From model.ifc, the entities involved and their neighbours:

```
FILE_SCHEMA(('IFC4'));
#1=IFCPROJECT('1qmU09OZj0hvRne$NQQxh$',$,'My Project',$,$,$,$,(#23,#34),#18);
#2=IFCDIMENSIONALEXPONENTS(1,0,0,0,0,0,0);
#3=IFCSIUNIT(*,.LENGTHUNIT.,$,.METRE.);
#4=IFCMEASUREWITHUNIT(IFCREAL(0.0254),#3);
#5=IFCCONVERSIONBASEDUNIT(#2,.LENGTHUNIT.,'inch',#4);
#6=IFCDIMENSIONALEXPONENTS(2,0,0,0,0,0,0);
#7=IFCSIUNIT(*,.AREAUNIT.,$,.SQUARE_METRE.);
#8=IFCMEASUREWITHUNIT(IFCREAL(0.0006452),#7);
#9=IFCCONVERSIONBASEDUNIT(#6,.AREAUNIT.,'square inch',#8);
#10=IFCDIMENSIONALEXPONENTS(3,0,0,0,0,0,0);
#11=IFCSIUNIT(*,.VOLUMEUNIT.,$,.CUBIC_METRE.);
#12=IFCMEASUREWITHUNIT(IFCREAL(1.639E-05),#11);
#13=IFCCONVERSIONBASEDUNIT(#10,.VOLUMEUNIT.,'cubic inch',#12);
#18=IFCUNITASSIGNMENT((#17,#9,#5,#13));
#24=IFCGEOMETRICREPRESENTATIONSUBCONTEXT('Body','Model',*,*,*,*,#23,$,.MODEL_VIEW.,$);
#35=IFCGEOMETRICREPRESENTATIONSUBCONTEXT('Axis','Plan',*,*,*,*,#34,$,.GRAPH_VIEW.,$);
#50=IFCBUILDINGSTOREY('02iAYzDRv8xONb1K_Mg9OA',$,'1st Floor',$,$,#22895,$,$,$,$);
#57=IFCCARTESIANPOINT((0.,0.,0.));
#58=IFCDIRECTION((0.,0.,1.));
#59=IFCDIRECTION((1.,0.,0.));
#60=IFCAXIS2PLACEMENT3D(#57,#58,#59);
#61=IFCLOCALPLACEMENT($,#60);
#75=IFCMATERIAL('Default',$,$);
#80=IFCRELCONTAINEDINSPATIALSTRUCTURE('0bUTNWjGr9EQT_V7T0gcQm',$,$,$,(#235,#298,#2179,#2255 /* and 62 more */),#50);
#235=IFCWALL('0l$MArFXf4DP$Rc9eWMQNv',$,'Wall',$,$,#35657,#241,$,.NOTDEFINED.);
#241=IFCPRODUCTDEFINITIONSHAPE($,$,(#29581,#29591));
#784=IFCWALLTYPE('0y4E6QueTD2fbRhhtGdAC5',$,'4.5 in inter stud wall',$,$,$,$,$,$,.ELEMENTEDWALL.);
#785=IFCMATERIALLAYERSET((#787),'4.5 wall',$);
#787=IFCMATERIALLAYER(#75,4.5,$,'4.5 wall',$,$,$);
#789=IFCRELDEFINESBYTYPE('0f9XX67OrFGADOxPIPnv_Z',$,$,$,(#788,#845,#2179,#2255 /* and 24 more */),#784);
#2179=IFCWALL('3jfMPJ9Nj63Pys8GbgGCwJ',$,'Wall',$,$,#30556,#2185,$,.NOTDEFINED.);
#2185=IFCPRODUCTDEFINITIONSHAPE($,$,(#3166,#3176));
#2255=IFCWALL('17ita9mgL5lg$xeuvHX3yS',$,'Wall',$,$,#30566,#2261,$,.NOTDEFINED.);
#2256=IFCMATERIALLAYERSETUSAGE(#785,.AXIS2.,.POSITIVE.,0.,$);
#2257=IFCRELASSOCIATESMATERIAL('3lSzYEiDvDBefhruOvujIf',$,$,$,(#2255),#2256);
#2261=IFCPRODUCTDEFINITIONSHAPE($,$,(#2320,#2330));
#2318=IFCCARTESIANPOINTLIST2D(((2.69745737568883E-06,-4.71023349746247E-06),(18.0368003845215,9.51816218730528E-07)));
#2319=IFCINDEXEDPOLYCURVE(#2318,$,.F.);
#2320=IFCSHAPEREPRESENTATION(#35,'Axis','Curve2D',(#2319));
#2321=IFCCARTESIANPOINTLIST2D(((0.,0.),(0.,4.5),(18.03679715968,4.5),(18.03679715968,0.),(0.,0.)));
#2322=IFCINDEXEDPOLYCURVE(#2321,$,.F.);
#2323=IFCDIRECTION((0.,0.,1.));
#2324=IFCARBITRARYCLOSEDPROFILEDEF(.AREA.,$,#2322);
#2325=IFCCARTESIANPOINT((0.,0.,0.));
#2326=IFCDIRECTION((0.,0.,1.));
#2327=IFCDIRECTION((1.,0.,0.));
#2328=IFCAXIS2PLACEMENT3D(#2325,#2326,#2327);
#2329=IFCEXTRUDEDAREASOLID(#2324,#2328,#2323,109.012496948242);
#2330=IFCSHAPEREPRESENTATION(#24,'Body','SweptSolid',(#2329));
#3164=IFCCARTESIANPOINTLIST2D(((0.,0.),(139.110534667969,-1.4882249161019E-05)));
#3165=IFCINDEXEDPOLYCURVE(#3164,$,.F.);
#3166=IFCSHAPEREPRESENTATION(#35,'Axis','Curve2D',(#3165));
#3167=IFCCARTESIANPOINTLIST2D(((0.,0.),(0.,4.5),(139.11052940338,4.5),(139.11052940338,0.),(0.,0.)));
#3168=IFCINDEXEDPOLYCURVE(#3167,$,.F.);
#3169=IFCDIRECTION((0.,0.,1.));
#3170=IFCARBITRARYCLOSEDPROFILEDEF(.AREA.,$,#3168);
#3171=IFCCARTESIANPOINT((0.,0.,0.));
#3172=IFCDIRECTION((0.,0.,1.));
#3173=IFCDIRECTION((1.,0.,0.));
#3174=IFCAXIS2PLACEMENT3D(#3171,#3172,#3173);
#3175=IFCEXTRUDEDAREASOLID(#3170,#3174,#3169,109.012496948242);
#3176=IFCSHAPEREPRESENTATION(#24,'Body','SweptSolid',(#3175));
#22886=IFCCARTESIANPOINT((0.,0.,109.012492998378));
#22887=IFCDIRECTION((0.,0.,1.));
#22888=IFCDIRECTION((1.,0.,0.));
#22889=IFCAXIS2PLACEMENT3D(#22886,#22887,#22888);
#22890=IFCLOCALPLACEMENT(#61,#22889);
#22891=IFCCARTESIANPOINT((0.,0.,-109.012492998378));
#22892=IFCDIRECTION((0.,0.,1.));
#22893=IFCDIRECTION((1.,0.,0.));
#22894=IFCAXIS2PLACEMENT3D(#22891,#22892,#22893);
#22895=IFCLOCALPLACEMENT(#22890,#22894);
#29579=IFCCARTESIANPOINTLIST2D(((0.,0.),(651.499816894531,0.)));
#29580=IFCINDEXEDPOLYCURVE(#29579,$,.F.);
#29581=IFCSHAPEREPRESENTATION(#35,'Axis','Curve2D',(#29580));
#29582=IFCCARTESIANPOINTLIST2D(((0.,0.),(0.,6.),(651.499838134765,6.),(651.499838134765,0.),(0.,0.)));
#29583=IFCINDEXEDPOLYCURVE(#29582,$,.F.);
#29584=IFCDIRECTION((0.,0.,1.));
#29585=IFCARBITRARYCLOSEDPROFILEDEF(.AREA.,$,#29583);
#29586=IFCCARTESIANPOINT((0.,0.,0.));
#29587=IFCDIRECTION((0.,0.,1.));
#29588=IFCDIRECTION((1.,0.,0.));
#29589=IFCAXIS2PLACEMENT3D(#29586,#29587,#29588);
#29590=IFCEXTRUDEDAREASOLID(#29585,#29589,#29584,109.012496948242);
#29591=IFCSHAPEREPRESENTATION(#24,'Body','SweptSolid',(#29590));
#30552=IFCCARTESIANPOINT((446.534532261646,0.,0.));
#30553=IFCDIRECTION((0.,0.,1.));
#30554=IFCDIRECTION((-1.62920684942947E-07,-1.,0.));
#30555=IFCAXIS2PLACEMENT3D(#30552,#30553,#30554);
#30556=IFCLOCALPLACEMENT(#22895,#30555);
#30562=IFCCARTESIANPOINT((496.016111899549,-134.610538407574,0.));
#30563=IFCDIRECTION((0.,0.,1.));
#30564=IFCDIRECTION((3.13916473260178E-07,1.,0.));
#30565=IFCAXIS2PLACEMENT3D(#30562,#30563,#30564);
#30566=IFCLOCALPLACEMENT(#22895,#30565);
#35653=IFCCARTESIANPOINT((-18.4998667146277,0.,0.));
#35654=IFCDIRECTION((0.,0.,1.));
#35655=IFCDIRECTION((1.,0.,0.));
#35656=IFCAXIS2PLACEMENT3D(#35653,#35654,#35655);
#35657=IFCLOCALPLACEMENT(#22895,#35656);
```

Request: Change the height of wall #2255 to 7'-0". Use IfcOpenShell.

```python
import ifcopenshell
import ifcopenshell.geom
import ifcopenshell.util.representation
import ifcopenshell.util.shape
import ifcopenshell.util.unit

model = ifcopenshell.open("model.ifc")
unit_scale = ifcopenshell.util.unit.calculate_unit_scale(model)
settings = ifcopenshell.geom.settings()


def volume(element):
    """Net volume in cubic metres, openings subtracted."""
    shape = ifcopenshell.geom.create_shape(settings, element)
    return ifcopenshell.util.shape.get_volume(shape.geometry)


wall = model.by_guid("17ita9mgL5lg$xeuvHX3yS")
before = volume(wall)

body = ifcopenshell.util.representation.get_representation(wall, "Model", "Body")
solid = body.Items[0]
old_height = solid.Depth
solid.Depth = 84 * 0.0254 / unit_scale
after = volume(wall)

print(f"height {old_height:g} -> {solid.Depth:g}, volume {before:.3f} -> {after:.3f} m3")

model.write("model_rev.ifc")
```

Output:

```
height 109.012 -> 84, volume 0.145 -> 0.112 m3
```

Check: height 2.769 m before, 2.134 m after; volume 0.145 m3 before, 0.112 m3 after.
